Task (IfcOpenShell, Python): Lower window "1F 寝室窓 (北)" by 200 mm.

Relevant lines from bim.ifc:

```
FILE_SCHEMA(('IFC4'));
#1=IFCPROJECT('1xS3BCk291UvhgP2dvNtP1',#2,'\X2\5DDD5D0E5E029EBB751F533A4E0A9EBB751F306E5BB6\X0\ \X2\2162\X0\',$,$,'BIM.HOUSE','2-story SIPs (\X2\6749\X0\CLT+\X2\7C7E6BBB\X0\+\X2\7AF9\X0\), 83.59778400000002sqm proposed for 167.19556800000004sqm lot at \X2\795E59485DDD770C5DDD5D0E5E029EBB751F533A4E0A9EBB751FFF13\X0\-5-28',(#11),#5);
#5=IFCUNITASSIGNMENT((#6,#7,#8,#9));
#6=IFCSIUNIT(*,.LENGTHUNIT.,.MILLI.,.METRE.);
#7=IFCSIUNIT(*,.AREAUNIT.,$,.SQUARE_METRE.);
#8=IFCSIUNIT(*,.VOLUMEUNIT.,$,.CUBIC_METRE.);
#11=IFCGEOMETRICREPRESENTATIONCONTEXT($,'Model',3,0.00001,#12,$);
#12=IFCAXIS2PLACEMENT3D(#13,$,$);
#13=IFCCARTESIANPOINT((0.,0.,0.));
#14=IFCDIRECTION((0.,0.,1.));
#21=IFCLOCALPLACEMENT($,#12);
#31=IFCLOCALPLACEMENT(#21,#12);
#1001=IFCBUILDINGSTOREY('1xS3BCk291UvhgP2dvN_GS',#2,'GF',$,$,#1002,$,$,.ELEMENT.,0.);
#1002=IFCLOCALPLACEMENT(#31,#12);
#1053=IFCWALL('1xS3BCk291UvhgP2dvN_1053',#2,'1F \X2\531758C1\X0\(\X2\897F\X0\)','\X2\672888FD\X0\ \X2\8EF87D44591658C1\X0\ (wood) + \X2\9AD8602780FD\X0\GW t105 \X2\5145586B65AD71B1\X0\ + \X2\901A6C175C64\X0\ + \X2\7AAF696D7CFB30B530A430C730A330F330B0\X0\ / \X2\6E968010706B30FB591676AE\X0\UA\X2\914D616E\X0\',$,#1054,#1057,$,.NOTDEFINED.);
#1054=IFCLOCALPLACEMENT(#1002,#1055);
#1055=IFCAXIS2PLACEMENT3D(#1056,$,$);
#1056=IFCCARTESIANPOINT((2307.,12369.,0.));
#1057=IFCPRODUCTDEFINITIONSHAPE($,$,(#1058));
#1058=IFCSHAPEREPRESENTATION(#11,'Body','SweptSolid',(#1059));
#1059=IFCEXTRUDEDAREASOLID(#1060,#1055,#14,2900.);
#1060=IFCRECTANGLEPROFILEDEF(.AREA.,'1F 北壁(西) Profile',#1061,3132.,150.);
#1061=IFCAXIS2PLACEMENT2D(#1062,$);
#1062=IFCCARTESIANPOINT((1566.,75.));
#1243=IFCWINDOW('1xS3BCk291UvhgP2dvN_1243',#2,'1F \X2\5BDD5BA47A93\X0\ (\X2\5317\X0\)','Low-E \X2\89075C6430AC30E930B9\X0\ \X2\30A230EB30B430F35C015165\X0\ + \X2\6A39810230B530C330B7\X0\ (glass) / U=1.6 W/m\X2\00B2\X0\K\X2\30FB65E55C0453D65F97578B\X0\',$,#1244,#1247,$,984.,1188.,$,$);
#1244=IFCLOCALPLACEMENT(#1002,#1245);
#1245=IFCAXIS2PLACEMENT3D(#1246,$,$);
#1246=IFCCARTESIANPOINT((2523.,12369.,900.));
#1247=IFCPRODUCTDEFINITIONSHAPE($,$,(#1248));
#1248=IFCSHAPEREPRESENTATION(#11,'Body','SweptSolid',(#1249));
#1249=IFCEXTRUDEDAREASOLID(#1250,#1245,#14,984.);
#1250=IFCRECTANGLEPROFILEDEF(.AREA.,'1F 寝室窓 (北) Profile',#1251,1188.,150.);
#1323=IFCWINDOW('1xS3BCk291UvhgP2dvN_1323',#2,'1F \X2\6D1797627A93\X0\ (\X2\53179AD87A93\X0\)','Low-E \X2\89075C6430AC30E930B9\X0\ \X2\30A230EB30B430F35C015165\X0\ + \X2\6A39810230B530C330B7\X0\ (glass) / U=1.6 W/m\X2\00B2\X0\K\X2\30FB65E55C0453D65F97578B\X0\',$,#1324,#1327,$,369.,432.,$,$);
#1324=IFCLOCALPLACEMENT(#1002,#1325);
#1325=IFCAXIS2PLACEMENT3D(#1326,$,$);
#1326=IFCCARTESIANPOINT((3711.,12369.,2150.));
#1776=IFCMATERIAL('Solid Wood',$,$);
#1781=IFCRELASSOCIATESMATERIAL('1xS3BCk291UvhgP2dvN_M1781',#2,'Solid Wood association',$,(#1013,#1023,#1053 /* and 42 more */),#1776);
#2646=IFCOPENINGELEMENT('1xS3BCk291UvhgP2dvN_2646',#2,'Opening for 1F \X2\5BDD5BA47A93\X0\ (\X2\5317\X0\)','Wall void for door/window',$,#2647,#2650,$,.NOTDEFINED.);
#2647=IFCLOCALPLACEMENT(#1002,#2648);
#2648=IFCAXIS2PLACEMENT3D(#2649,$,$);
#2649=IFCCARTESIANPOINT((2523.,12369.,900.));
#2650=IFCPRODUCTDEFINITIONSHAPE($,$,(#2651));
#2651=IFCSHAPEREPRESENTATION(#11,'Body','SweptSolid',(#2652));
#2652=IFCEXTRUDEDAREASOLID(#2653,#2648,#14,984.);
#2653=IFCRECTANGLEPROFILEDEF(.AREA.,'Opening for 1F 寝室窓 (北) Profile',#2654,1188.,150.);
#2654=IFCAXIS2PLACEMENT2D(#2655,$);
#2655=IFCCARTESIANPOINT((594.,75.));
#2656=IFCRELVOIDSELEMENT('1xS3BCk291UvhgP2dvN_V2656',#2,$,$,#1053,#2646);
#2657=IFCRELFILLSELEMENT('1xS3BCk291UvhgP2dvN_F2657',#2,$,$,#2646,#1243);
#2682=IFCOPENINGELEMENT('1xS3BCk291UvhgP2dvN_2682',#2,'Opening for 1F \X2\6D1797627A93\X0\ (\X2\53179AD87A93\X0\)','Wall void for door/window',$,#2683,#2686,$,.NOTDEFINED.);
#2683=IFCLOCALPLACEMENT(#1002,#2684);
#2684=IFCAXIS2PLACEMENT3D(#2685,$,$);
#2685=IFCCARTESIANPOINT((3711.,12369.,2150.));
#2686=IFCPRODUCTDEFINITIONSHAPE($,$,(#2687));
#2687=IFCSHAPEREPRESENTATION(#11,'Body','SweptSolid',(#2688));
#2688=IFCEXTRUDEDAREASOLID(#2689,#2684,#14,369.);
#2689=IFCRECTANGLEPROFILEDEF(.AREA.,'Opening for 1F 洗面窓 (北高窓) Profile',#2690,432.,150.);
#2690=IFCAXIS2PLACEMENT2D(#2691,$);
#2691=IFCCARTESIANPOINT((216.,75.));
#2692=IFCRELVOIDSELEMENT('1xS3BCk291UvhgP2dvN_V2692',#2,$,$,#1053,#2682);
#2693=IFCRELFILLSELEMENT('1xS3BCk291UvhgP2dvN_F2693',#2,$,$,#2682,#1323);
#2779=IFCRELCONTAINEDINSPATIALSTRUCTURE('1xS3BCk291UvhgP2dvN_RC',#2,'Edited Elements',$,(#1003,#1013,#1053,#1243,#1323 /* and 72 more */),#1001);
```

```python
import numpy as np
import ifcopenshell
import ifcopenshell.api.geometry
import ifcopenshell.util.placement
import ifcopenshell.util.unit

model = ifcopenshell.open("bim.ifc")
unit_scale = ifcopenshell.util.unit.calculate_unit_scale(model)

window = model.by_guid("1xS3BCk291UvhgP2dvN_1243")
opening = window.FillsVoids[0].RelatingOpeningElement
dz = -0.2 / unit_scale

shift = np.array([0.0, 0.0, dz])
# The window is not placed relative to its opening, so move both.
for product in (opening, window):
    matrix = ifcopenshell.util.placement.get_local_placement(product.ObjectPlacement)
    matrix[:3, 3] += shift
    ifcopenshell.api.geometry.edit_object_placement(model, product=product, matrix=matrix, is_si=False)

print(f"moved by {dz * unit_scale:+.3f} m")

model.write("bim_edited.ifc")
```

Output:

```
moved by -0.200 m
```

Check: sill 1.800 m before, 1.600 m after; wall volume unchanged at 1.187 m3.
